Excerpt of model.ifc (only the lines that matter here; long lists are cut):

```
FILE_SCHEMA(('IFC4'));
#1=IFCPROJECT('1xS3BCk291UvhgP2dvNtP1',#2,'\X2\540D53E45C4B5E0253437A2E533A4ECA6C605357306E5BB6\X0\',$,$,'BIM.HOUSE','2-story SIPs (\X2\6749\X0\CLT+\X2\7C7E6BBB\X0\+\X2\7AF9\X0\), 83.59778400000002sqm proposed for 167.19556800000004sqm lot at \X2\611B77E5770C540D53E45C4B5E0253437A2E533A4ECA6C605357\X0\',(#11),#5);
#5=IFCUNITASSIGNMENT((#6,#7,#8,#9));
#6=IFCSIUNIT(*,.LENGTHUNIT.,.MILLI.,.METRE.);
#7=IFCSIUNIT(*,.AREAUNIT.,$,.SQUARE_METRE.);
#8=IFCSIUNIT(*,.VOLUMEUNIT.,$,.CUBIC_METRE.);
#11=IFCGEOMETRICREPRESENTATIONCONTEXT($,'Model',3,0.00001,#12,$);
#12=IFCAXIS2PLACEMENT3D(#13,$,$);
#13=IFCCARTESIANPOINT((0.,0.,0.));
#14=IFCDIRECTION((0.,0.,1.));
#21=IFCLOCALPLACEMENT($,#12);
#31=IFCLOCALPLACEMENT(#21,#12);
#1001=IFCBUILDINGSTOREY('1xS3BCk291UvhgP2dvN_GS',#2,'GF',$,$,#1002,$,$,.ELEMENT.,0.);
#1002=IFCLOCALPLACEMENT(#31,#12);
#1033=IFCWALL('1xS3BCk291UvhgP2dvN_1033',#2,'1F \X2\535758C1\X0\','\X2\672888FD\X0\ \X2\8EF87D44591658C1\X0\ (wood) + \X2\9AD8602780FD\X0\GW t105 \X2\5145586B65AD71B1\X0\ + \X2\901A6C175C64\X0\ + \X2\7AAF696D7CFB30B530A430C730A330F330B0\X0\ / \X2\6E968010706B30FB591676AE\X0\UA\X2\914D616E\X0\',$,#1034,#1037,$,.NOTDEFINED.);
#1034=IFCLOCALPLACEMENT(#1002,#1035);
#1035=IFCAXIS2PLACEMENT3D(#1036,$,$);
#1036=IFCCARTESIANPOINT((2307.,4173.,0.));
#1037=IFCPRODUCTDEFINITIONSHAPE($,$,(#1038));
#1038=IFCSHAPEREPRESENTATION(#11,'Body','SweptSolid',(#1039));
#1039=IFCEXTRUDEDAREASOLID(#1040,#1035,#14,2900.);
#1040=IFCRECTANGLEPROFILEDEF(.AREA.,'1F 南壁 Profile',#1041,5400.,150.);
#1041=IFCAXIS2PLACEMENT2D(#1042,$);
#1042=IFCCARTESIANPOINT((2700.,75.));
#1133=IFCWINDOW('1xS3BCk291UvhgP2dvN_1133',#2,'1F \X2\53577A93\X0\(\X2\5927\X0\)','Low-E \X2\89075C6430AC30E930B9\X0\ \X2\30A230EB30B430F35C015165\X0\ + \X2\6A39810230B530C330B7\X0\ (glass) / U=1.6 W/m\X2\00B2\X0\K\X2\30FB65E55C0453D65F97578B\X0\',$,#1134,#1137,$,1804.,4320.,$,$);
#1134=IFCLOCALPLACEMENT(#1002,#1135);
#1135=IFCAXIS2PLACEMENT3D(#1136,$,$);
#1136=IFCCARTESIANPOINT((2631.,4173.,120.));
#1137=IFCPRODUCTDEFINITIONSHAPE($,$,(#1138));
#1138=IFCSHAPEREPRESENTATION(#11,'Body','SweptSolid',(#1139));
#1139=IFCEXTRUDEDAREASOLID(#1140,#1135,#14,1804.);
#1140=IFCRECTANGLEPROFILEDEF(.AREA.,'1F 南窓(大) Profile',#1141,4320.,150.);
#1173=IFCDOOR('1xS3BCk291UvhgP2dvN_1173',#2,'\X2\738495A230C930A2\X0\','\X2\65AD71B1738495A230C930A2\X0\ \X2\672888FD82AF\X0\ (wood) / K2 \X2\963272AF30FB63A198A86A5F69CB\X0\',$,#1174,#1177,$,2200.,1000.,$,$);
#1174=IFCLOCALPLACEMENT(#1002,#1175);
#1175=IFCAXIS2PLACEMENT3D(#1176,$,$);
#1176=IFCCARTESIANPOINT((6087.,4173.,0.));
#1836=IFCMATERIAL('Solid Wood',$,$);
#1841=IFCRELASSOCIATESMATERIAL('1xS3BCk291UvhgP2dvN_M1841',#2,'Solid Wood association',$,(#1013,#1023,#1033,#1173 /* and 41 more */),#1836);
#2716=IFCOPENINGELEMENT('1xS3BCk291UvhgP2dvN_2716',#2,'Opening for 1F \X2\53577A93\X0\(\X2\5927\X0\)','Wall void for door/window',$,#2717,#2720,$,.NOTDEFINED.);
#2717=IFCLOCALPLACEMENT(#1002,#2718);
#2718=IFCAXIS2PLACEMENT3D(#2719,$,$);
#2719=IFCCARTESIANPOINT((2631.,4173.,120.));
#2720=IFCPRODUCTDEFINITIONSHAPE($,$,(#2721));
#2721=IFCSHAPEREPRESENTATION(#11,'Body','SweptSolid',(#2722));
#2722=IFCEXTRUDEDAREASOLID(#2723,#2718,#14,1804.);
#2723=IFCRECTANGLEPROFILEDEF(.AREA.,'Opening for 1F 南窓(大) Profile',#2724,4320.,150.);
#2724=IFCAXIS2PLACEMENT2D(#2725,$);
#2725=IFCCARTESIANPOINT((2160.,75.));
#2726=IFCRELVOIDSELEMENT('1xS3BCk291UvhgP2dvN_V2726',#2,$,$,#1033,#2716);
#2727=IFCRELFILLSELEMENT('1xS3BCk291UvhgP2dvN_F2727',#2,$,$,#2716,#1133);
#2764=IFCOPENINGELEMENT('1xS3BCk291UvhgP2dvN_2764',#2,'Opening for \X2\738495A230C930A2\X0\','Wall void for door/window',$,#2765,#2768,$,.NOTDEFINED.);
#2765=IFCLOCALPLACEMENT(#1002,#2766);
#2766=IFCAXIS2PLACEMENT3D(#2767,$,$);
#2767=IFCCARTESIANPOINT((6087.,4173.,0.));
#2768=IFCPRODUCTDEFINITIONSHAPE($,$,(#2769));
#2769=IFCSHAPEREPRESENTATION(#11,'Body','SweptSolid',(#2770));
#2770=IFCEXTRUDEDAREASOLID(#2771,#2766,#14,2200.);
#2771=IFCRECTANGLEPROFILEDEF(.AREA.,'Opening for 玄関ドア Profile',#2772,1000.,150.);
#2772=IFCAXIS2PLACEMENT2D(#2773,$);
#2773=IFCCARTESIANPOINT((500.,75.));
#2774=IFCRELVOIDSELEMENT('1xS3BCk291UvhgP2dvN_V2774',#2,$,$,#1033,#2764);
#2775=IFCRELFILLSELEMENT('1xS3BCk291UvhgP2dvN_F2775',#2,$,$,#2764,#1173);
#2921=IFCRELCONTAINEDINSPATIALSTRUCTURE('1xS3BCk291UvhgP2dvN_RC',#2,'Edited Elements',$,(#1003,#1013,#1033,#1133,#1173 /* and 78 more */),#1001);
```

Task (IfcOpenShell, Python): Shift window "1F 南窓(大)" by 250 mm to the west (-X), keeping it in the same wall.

```python
import ifcopenshell
import ifcopenshell.api.geometry
import ifcopenshell.util.placement
import ifcopenshell.util.unit

model = ifcopenshell.open("model.ifc")
unit_scale = ifcopenshell.util.unit.calculate_unit_scale(model)

window = model.by_guid("1xS3BCk291UvhgP2dvN_1133")
opening = window.FillsVoids[0].RelatingOpeningElement
wall = opening.VoidsElements[0].RelatingBuildingElement

wall_matrix = ifcopenshell.util.placement.get_local_placement(wall.ObjectPlacement)
shift = wall_matrix[:3, 0] * -0.25 / unit_scale
before = ifcopenshell.util.placement.get_local_placement(window.ObjectPlacement)[:3, 3].copy()

# The window is not placed relative to its opening, so move both.
for product in (opening, window):
    matrix = ifcopenshell.util.placement.get_local_placement(product.ObjectPlacement)
    matrix[:3, 3] += shift
    ifcopenshell.api.geometry.edit_object_placement(model, product=product, matrix=matrix, is_si=False)

after = ifcopenshell.util.placement.get_local_placement(window.ObjectPlacement)[:3, 3]
print("window moved by", (after - before).round(3) + 0.0)

model.write("model_v2.ifc")
```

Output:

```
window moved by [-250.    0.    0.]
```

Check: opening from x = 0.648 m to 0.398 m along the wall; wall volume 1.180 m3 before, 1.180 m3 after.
